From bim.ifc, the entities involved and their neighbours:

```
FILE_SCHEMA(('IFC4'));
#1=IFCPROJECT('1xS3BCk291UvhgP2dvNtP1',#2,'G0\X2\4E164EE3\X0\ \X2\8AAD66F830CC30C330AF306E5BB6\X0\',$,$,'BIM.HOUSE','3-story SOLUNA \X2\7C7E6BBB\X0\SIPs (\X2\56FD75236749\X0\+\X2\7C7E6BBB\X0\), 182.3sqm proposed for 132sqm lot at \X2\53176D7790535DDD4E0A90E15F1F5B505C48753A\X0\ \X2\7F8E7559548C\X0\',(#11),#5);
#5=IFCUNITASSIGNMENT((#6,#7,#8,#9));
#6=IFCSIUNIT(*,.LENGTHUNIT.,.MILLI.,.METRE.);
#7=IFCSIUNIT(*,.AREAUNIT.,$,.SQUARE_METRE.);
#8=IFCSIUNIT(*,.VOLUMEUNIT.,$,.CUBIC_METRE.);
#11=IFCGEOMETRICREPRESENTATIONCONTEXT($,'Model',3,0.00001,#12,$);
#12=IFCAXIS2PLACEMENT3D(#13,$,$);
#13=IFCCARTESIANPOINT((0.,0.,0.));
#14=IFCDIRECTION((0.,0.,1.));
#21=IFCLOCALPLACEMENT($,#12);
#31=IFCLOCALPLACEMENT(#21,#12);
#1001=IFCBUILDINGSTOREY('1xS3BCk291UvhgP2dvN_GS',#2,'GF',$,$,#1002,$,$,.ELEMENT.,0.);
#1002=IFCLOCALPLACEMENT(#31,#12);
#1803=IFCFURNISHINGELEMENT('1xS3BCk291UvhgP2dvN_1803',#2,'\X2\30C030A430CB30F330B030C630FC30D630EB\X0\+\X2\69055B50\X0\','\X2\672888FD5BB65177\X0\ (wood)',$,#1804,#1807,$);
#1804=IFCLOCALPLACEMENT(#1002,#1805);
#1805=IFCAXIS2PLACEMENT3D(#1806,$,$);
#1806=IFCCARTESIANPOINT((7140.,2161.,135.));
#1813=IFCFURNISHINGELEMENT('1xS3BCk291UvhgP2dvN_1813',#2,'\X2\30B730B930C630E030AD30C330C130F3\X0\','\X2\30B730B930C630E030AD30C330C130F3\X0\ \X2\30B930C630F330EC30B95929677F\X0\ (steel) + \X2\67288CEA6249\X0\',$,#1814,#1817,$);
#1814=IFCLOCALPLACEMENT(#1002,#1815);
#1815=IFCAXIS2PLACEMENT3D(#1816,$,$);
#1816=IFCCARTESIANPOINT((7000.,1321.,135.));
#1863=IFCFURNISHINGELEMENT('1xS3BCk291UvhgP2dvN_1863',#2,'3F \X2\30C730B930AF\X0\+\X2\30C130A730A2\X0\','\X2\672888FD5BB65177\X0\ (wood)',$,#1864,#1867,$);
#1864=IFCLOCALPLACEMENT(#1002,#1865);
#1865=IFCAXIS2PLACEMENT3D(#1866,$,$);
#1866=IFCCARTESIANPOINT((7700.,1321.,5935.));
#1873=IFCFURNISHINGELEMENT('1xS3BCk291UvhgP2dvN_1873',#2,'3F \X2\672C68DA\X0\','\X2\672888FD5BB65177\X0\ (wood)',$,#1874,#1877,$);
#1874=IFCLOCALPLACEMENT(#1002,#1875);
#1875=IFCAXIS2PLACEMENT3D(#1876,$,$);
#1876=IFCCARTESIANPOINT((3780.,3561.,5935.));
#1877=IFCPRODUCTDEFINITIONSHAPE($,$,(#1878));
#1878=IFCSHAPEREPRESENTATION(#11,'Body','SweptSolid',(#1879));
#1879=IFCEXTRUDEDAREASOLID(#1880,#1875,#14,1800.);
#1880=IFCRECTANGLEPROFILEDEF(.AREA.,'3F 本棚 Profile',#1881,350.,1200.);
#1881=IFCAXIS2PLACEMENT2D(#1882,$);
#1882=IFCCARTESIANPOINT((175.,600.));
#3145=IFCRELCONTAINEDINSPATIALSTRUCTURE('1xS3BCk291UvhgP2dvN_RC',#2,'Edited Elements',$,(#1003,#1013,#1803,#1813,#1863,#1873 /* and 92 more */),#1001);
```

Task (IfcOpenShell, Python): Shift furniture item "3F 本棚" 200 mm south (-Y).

```python
import ifcopenshell
import ifcopenshell.api.geometry
import ifcopenshell.util.placement
import ifcopenshell.util.unit

model = ifcopenshell.open("bim.ifc")
unit_scale = ifcopenshell.util.unit.calculate_unit_scale(model)

item = model.by_guid("1xS3BCk291UvhgP2dvN_1873")
matrix = ifcopenshell.util.placement.get_local_placement(item.ObjectPlacement)
matrix[1, 3] -= 0.2 / unit_scale
ifcopenshell.api.geometry.edit_object_placement(model, product=item, matrix=matrix, is_si=False)

print(ifcopenshell.util.placement.get_local_placement(item.ObjectPlacement).round(3) + 0.0)

model.write("bim_edited.ifc")
```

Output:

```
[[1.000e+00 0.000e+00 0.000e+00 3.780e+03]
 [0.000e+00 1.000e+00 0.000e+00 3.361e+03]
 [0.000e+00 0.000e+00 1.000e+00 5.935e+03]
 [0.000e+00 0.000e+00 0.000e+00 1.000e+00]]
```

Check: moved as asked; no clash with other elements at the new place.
